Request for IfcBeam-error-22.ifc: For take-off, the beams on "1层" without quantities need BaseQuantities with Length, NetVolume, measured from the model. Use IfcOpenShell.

First a look at what the model holds.

```python
import ifcopenshell
import ifcopenshell.util.element
import ifcopenshell.util.unit

model = ifcopenshell.open("IfcBeam-error-22.ifc")
print(model.schema)
for unit_type in ("LENGTHUNIT", "AREAUNIT", "VOLUMEUNIT"):
    print(unit_type, ifcopenshell.util.unit.calculate_unit_scale(model, unit_type))
storey = next(s for s in model.by_type("IfcBuildingStorey") if s.Name == "1层")
beams = [e for e in ifcopenshell.util.element.get_decomposition(storey) if e.is_a("IfcBeam")]
for e in sorted(beams, key=lambda e: e.id()):
    print(e.id(), e.is_a(), e.Name, list(ifcopenshell.util.element.get_psets(e, qtos_only=True)), sep=" | ")
```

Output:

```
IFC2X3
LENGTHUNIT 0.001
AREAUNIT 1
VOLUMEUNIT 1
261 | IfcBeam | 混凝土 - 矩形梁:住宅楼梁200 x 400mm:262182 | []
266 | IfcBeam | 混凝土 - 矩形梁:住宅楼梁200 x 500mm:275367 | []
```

```python
import ifcopenshell
import ifcopenshell.api.pset
import ifcopenshell.geom
import ifcopenshell.util.element
import ifcopenshell.util.shape
import ifcopenshell.util.unit

model = ifcopenshell.open("IfcBeam-error-22.ifc")
unit_scale = ifcopenshell.util.unit.calculate_unit_scale(model)
volume_scale = ifcopenshell.util.unit.calculate_unit_scale(model, "VOLUMEUNIT")
settings = ifcopenshell.geom.settings()

storey = next(s for s in model.by_type("IfcBuildingStorey") if s.Name == "1层")
beams = [e for e in ifcopenshell.util.element.get_decomposition(storey) if e.is_a("IfcBeam")]

for e in sorted(beams, key=lambda e: e.id()):
    if ifcopenshell.util.element.get_psets(e, qtos_only=True, should_inherit=False):
        continue
    # Geometry comes back in metres, in the element's own axes.
    shape = ifcopenshell.geom.create_shape(settings, e)
    values = {
        "Length": ifcopenshell.util.shape.get_max_xyz(shape.geometry) / unit_scale,
        "NetVolume": ifcopenshell.util.shape.get_volume(shape.geometry) / volume_scale,
    }
    qto = ifcopenshell.api.pset.add_qto(model, product=e, name="BaseQuantities")
    ifcopenshell.api.pset.edit_qto(model, qto=qto, properties=values)
    print(e.id(), {k: round(v, 3) for k, v in values.items()})

model.write("IfcBeam-error-22_v2.ifc")
```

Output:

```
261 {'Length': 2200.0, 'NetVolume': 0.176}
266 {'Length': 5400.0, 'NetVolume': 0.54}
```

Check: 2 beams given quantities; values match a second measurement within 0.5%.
